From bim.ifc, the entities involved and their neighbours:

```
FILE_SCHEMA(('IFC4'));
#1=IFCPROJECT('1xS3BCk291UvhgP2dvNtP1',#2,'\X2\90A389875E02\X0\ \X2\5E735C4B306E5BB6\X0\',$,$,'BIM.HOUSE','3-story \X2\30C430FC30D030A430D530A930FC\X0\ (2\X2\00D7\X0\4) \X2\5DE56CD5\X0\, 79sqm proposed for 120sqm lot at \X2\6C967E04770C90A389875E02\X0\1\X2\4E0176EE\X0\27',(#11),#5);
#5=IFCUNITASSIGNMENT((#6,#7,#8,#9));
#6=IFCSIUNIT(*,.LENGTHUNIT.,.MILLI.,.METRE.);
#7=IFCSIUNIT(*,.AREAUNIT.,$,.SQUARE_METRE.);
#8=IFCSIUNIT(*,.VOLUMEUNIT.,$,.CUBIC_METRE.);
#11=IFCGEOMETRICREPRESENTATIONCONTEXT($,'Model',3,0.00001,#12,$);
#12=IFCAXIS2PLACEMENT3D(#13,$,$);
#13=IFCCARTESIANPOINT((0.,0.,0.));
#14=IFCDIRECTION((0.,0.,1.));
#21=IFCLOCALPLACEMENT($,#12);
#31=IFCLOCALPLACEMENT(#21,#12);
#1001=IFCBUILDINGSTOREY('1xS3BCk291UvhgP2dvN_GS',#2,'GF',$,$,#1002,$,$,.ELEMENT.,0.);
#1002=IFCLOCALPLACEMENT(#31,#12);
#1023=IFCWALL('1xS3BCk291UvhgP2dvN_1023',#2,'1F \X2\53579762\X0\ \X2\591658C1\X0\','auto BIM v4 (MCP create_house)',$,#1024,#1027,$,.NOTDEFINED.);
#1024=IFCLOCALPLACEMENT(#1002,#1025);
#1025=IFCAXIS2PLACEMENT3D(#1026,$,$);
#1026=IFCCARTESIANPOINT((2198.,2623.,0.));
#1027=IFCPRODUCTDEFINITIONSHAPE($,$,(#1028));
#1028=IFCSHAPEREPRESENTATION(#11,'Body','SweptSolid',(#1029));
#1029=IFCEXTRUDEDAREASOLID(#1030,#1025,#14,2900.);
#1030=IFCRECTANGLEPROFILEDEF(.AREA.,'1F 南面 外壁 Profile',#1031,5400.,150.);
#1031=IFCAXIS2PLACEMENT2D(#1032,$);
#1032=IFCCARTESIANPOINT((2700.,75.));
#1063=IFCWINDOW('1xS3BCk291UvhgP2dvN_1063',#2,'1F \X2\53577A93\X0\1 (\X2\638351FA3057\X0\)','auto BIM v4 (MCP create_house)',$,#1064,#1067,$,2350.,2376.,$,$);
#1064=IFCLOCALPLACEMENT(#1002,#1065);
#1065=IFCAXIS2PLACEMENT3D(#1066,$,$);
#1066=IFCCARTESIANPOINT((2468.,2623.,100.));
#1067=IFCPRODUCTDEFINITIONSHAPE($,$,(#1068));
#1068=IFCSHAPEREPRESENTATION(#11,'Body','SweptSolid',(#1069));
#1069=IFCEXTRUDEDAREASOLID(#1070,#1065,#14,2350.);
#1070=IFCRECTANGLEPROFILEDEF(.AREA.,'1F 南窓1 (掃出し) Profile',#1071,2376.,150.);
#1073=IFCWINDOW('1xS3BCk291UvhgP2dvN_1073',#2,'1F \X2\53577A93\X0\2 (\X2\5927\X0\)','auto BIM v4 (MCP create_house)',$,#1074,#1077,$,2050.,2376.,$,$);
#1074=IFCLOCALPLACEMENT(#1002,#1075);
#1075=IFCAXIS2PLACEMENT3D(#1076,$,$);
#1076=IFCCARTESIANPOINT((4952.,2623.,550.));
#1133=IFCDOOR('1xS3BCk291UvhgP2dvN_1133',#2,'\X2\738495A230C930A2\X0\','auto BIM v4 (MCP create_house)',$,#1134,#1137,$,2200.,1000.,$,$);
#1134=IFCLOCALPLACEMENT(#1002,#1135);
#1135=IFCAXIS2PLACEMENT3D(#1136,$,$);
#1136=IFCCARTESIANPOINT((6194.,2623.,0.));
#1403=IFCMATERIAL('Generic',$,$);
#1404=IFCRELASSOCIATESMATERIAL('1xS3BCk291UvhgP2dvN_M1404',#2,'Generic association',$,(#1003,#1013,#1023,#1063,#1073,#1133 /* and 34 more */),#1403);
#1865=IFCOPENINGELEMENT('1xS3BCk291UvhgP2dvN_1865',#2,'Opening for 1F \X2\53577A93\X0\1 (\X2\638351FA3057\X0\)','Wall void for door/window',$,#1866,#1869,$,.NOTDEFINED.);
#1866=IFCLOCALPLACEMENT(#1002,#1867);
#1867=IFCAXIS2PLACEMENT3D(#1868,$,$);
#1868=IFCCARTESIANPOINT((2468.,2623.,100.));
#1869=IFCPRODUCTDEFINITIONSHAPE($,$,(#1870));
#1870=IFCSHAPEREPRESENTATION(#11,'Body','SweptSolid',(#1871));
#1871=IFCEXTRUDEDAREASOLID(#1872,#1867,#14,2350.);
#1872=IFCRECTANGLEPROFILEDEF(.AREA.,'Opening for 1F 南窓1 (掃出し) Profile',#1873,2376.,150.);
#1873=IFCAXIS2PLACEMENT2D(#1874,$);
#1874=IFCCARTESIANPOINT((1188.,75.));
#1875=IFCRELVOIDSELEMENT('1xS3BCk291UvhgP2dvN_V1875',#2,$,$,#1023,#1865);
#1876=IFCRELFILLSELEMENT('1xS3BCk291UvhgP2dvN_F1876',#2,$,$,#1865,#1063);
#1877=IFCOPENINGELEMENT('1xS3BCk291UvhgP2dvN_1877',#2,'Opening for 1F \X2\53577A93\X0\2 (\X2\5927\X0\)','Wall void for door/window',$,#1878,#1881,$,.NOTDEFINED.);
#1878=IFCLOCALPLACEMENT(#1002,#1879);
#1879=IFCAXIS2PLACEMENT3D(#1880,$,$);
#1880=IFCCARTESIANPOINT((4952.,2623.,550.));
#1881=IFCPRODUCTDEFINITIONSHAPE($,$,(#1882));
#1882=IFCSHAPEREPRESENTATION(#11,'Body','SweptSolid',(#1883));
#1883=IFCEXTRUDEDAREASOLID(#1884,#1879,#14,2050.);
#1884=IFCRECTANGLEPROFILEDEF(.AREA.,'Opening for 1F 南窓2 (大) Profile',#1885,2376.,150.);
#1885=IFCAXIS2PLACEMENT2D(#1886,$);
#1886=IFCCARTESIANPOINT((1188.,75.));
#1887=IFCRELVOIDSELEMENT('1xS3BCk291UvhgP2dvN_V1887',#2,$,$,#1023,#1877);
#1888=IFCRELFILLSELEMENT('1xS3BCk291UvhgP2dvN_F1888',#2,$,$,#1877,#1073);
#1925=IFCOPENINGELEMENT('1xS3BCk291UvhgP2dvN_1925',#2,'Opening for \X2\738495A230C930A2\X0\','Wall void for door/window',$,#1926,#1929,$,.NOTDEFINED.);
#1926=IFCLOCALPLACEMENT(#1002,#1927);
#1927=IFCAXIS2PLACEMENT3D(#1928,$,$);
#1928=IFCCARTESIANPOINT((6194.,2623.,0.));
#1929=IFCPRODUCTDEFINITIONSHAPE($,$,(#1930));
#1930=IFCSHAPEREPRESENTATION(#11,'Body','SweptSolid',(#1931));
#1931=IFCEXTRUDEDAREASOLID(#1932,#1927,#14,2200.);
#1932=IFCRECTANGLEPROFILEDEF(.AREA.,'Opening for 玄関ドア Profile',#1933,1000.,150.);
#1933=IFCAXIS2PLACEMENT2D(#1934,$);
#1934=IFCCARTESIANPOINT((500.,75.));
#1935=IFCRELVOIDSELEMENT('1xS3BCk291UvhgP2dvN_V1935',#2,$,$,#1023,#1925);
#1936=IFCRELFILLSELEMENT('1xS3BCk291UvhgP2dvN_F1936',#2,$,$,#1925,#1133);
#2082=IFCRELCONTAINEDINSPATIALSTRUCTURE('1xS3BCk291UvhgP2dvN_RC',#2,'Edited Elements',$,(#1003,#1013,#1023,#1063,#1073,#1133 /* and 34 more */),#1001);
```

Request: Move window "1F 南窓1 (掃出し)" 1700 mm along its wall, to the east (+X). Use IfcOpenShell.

```python
import ifcopenshell
import ifcopenshell.api.geometry
import ifcopenshell.util.placement

model = ifcopenshell.open("bim.ifc")

window = model.by_guid("1xS3BCk291UvhgP2dvN_1063")
opening = window.FillsVoids[0].RelatingOpeningElement
wall = opening.VoidsElements[0].RelatingBuildingElement

wall_matrix = ifcopenshell.util.placement.get_local_placement(wall.ObjectPlacement)
shift = wall_matrix[:3, 0] * 1700.0
before = ifcopenshell.util.placement.get_local_placement(window.ObjectPlacement)[:3, 3].copy()

# The window is not placed relative to its opening, so move both.
for product in (opening, window):
    matrix = ifcopenshell.util.placement.get_local_placement(product.ObjectPlacement)
    matrix[:3, 3] += shift
    ifcopenshell.api.geometry.edit_object_placement(model, product=product, matrix=matrix, is_si=False)

after = ifcopenshell.util.placement.get_local_placement(window.ObjectPlacement)[:3, 3]
print("window moved by", (after - before).round(3) + 0.0)

model.write("bim_updated.ifc")
```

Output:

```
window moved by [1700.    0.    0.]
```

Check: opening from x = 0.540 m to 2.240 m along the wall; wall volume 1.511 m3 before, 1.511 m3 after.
